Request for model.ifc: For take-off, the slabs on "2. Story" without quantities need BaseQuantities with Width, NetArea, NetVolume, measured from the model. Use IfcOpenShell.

First a look at what the model holds.

```python
import ifcopenshell
import ifcopenshell.util.element
import ifcopenshell.util.unit

model = ifcopenshell.open("model.ifc")
print(model.schema)
for unit_type in ("LENGTHUNIT", "AREAUNIT", "VOLUMEUNIT"):
    print(unit_type, ifcopenshell.util.unit.calculate_unit_scale(model, unit_type))
storey = next(s for s in model.by_type("IfcBuildingStorey") if s.Name == "2. Story")
slabs = [e for e in ifcopenshell.util.element.get_decomposition(storey) if e.is_a("IfcSlab")]
for e in sorted(slabs, key=lambda e: e.id()):
    print(e.id(), e.is_a(), e.Name, list(ifcopenshell.util.element.get_psets(e, qtos_only=True)), sep=" | ")
```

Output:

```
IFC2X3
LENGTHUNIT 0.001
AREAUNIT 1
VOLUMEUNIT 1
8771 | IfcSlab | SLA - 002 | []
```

```python
import ifcopenshell
import ifcopenshell.api.pset
import ifcopenshell.geom
import ifcopenshell.util.element
import ifcopenshell.util.shape
import ifcopenshell.util.unit

model = ifcopenshell.open("model.ifc")
unit_scale = ifcopenshell.util.unit.calculate_unit_scale(model)
area_scale = ifcopenshell.util.unit.calculate_unit_scale(model, "AREAUNIT")
volume_scale = ifcopenshell.util.unit.calculate_unit_scale(model, "VOLUMEUNIT")
settings = ifcopenshell.geom.settings()

storey = next(s for s in model.by_type("IfcBuildingStorey") if s.Name == "2. Story")
slabs = [e for e in ifcopenshell.util.element.get_decomposition(storey) if e.is_a("IfcSlab")]

for e in sorted(slabs, key=lambda e: e.id()):
    if ifcopenshell.util.element.get_psets(e, qtos_only=True, should_inherit=False):
        continue
    # Geometry comes back in metres, in the element's own axes.
    shape = ifcopenshell.geom.create_shape(settings, e)
    values = {
        "Width": ifcopenshell.util.shape.get_z(shape.geometry) / unit_scale,
        "NetArea": ifcopenshell.util.shape.get_footprint_area(shape.geometry) / area_scale,
        "NetVolume": ifcopenshell.util.shape.get_volume(shape.geometry) / volume_scale,
    }
    qto = ifcopenshell.api.pset.add_qto(model, product=e, name="BaseQuantities")
    ifcopenshell.api.pset.edit_qto(model, qto=qto, properties=values)
    print(e.id(), {k: round(v, 3) for k, v in values.items()})

model.write("model_updated.ifc")
```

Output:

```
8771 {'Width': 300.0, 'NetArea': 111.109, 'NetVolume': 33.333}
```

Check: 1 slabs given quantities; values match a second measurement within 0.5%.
